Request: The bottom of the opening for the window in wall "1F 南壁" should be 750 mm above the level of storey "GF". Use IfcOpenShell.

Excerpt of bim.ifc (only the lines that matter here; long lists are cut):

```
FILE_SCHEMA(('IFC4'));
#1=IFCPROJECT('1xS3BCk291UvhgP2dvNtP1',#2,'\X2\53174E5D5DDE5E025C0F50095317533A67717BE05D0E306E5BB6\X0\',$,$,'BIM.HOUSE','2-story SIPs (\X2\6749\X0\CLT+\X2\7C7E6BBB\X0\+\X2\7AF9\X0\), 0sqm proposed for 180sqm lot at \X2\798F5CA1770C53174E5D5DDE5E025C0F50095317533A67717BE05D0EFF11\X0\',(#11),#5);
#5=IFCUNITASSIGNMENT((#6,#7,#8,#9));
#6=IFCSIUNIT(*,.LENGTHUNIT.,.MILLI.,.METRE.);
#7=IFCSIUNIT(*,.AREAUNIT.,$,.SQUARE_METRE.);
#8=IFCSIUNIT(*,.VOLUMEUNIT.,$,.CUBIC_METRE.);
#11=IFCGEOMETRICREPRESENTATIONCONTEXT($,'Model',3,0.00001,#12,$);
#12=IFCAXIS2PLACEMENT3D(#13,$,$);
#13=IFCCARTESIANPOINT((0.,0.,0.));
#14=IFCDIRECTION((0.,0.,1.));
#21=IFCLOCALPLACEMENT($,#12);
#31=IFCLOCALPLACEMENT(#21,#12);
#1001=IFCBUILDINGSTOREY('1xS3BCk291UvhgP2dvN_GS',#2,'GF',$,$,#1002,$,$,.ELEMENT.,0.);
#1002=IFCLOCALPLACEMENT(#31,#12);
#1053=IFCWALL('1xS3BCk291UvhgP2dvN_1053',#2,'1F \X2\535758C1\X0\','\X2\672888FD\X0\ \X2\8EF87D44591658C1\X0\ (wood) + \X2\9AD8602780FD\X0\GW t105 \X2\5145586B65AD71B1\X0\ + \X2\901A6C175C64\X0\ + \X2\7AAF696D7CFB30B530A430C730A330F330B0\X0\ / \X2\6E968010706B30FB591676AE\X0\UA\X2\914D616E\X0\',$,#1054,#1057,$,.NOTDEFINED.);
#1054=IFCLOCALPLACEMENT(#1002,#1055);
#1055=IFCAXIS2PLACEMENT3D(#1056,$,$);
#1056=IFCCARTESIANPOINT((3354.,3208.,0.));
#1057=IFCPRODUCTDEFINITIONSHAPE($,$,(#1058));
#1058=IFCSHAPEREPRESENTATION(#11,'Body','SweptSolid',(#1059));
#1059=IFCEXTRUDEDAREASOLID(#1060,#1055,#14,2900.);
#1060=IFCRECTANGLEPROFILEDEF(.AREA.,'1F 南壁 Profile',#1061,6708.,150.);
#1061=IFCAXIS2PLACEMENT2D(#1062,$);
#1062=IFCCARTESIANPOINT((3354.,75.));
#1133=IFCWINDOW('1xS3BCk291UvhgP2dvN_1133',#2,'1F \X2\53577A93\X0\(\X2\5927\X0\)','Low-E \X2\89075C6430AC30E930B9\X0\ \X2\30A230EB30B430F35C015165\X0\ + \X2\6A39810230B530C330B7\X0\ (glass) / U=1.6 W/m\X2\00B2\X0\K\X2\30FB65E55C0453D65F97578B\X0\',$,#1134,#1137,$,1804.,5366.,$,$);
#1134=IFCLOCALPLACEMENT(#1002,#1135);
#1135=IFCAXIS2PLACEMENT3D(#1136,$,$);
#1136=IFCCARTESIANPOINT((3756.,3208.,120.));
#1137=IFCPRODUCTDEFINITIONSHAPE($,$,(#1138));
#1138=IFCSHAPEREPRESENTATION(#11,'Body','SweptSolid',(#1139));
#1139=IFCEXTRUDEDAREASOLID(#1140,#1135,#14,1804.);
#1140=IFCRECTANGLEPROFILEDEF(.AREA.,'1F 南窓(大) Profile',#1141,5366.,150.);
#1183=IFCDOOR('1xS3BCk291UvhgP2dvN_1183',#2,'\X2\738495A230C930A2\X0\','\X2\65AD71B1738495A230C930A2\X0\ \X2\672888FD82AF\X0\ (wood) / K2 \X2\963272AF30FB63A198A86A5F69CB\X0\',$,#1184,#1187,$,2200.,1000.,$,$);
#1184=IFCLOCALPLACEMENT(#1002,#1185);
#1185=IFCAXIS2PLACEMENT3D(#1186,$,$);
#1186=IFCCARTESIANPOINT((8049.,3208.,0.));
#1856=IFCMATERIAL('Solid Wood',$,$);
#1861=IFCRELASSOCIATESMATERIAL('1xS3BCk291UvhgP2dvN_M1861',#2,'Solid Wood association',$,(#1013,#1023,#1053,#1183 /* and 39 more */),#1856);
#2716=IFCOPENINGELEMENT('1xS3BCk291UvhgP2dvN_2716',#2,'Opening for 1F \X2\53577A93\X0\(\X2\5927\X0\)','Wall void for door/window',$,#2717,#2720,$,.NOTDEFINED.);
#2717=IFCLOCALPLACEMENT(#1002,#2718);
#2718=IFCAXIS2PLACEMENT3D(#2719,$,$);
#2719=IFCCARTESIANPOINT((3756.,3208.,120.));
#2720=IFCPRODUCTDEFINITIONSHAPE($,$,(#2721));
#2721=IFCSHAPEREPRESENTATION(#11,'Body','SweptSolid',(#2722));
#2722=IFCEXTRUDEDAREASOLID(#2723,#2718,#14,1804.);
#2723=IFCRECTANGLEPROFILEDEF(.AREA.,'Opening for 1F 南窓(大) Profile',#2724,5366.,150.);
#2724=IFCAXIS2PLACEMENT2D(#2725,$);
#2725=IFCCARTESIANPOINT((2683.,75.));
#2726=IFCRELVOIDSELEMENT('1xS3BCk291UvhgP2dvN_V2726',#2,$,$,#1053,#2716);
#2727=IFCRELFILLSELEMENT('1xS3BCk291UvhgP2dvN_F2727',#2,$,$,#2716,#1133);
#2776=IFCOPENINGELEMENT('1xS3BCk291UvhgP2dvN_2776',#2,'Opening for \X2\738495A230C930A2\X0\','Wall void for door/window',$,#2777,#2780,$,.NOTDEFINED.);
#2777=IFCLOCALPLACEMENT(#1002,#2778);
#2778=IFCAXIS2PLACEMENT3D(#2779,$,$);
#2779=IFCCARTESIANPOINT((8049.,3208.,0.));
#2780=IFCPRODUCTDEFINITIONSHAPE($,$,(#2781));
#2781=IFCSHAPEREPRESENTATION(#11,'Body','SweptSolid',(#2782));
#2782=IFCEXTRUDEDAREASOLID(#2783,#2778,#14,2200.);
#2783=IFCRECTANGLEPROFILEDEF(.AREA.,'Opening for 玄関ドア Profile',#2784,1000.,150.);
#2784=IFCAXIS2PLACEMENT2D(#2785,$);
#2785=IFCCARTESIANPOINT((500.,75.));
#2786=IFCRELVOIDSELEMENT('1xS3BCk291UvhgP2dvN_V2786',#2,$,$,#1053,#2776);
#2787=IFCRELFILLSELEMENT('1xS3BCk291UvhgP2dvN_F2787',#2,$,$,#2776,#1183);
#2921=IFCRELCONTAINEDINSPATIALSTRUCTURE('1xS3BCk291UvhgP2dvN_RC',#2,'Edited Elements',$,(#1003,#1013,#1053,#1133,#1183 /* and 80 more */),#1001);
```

```python
import numpy as np
import ifcopenshell
import ifcopenshell.api.geometry
import ifcopenshell.geom
import ifcopenshell.util.element
import ifcopenshell.util.placement
import ifcopenshell.util.shape
import ifcopenshell.util.unit

model = ifcopenshell.open("bim.ifc")
unit_scale = ifcopenshell.util.unit.calculate_unit_scale(model)

window = model.by_guid("1xS3BCk291UvhgP2dvN_1133")
opening = window.FillsVoids[0].RelatingOpeningElement
storey = ifcopenshell.util.element.get_container(window, ifc_class="IfcBuildingStorey")
level = ifcopenshell.util.placement.get_local_placement(storey.ObjectPlacement)[2, 3]

# The opening's origin need not be at the sill, so measure its lowest point.
shape = ifcopenshell.geom.create_shape(ifcopenshell.geom.settings(), opening)
bottom = ifcopenshell.util.shape.get_shape_bottom_elevation(shape, shape.geometry) / unit_scale
dz = level + 0.75 / unit_scale - bottom

shift = np.array([0.0, 0.0, dz])
# The window is not placed relative to its opening, so move both.
for product in (opening, window):
    matrix = ifcopenshell.util.placement.get_local_placement(product.ObjectPlacement)
    matrix[:3, 3] += shift
    ifcopenshell.api.geometry.edit_object_placement(model, product=product, matrix=matrix, is_si=False)

print(f"moved by {dz * unit_scale:+.3f} m")

model.write("bim_edited.ifc")
```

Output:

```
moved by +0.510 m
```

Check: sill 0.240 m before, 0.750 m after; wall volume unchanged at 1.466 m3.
